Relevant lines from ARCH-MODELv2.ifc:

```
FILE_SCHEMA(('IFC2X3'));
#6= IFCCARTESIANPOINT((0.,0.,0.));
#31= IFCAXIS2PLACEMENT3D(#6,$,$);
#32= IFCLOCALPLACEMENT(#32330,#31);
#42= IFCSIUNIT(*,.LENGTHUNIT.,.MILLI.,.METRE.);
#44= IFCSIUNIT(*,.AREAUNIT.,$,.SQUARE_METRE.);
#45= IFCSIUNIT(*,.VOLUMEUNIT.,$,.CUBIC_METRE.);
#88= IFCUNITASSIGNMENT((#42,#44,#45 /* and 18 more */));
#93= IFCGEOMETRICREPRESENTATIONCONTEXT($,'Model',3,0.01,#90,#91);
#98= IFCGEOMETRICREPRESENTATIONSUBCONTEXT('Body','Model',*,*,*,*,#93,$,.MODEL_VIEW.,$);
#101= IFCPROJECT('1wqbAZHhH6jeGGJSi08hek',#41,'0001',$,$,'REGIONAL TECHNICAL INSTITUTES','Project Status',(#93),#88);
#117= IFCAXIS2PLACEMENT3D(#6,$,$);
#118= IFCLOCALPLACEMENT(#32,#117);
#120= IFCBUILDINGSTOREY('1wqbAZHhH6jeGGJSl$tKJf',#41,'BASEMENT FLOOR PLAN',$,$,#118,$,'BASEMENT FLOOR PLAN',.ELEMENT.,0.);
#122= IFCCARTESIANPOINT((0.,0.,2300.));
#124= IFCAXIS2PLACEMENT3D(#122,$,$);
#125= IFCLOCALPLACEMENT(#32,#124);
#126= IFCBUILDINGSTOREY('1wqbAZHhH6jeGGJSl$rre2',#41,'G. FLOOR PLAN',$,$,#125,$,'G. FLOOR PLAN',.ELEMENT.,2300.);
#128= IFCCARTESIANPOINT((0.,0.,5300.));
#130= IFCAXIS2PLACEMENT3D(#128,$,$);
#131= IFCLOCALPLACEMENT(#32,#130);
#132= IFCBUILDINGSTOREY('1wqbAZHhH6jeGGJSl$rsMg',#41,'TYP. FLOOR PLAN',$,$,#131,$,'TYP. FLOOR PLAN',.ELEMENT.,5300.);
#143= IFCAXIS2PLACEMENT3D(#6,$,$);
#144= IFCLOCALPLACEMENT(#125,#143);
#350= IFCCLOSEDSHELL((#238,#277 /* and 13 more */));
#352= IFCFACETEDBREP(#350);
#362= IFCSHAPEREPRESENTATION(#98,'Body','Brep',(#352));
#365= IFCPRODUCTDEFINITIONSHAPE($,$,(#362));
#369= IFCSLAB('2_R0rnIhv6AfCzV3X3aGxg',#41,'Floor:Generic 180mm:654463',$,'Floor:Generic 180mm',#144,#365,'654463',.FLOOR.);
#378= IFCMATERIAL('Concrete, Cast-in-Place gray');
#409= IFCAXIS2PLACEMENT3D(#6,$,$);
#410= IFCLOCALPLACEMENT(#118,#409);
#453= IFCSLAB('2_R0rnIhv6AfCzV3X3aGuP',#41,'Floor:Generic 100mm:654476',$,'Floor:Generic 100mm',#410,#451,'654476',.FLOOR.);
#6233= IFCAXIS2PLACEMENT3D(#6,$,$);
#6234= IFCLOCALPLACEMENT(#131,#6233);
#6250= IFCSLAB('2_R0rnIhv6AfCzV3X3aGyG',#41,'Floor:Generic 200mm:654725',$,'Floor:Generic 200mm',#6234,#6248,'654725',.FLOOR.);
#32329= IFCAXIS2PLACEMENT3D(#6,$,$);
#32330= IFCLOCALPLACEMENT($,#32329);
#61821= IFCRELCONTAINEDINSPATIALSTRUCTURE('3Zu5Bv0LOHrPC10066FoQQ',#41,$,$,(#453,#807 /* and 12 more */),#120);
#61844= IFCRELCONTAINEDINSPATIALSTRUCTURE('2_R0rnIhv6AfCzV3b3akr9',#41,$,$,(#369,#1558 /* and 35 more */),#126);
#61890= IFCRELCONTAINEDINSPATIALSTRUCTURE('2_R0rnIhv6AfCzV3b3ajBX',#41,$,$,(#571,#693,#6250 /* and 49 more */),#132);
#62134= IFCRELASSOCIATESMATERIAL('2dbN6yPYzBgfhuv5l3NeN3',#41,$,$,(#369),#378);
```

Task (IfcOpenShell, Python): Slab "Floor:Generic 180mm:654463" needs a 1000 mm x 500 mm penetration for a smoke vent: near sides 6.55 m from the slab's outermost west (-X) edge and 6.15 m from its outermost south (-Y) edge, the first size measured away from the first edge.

```python
import numpy as np
import ifcopenshell
import ifcopenshell.api.feature
import ifcopenshell.api.geometry
import ifcopenshell.api.root
import ifcopenshell.geom
import ifcopenshell.util.placement
import ifcopenshell.util.representation
import ifcopenshell.util.shape
import ifcopenshell.util.unit

model = ifcopenshell.open("ARCH-MODELv2.ifc")
unit_scale = ifcopenshell.util.unit.calculate_unit_scale(model)
settings = ifcopenshell.geom.settings()


def volume(element):
    """Net volume in cubic metres, openings subtracted."""
    shape = ifcopenshell.geom.create_shape(settings, element)
    return ifcopenshell.util.shape.get_volume(shape.geometry)


slab = model.by_id(369)
before = volume(slab)

# Extent in the slab's own axes, in metres. The edges named are its -X and -Y sides.
slab_shape = ifcopenshell.geom.create_shape(settings, slab)
vertices = ifcopenshell.util.shape.get_vertices(slab_shape.geometry)
x_min, y_min, bottom = vertices.min(axis=0)
top = vertices[:, 2].max()

opening = ifcopenshell.api.root.create_entity(model, ifc_class="IfcOpeningElement", name="Smoke vent opening")
context = ifcopenshell.util.representation.get_context(model, "Model", "Body", "MODEL_VIEW")
width, depth = 1, 0.5
outline = [(0.0, 0.0), (width, 0.0), (width, depth), (0.0, depth), (0.0, 0.0)]
# Overshoot both faces by 50 mm so the cut is clean.
shape = ifcopenshell.api.geometry.add_slab_representation(
    model, context=context, depth=top - bottom + 0.1, polyline=outline
)
ifcopenshell.api.geometry.assign_representation(model, product=opening, representation=shape)

matrix = ifcopenshell.util.placement.get_local_placement(slab.ObjectPlacement)
matrix[:, 3] = matrix @ np.append(np.array([x_min + 6.55, y_min + 6.15, bottom - 0.05]) / unit_scale, 1.0)
ifcopenshell.api.geometry.edit_object_placement(model, product=opening, matrix=matrix, is_si=False)
ifcopenshell.api.feature.add_feature(model, feature=opening, element=slab)

after = volume(slab)

print(f"slab volume {before:.3f} -> {after:.3f} m3")

model.write("ARCH-MODELv2_updated.ifc")
```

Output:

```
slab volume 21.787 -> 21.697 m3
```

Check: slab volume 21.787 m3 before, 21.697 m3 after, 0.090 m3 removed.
